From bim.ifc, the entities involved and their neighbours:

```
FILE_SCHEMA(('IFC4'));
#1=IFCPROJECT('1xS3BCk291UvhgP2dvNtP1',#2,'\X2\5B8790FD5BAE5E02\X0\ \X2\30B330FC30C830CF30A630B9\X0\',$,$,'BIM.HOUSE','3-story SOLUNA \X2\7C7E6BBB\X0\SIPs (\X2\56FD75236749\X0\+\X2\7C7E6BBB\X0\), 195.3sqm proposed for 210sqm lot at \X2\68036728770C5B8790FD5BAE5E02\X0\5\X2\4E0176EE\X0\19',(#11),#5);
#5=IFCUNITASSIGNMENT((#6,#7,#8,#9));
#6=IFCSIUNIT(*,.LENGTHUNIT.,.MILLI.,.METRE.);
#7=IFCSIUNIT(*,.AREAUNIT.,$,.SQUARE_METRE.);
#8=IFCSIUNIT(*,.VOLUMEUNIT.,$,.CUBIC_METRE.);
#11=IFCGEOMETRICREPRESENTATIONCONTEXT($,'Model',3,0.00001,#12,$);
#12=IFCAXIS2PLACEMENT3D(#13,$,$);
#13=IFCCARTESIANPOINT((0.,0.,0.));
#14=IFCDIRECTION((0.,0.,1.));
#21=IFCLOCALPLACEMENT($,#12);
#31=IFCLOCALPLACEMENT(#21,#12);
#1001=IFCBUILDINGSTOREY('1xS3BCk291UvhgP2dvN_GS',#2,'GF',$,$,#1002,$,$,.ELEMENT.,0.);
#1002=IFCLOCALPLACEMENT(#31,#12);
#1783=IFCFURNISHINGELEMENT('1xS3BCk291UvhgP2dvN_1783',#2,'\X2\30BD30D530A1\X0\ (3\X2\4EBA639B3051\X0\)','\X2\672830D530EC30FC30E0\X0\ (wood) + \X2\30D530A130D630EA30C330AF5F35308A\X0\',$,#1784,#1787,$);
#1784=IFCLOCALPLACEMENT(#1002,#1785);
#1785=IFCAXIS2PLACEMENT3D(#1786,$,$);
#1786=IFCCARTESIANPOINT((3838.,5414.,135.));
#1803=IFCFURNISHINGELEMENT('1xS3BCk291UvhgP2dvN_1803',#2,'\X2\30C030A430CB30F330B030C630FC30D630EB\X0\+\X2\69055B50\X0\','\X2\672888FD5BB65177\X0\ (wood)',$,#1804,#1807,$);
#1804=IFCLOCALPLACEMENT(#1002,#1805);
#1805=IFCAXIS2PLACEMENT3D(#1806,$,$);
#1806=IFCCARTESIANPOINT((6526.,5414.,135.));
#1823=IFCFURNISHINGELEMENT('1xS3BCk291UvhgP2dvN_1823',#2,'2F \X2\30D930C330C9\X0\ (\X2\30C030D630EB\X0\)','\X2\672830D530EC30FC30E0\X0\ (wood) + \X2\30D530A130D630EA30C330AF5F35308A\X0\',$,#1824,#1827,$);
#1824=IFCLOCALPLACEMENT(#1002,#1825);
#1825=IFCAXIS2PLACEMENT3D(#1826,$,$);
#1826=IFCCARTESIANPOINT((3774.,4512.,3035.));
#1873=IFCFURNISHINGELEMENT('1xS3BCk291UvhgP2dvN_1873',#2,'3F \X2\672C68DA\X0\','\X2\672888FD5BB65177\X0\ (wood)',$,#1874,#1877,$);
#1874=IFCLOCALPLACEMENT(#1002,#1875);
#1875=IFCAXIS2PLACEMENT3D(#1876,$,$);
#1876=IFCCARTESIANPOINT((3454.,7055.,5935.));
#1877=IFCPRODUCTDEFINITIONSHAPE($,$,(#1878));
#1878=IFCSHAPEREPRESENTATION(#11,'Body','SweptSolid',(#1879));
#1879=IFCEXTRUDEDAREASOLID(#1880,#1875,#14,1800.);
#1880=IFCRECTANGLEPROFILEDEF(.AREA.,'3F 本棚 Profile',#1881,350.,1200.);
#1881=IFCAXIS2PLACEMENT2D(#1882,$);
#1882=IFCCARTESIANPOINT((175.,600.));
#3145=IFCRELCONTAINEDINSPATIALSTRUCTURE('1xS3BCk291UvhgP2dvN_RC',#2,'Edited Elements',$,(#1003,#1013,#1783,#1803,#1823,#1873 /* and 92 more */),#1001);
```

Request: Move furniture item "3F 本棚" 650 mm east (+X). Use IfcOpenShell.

```python
import ifcopenshell
import ifcopenshell.api.geometry
import ifcopenshell.util.placement
import ifcopenshell.util.unit

model = ifcopenshell.open("bim.ifc")
unit_scale = ifcopenshell.util.unit.calculate_unit_scale(model)

item = model.by_id(1873)
matrix = ifcopenshell.util.placement.get_local_placement(item.ObjectPlacement)
matrix[0, 3] += 0.65 / unit_scale
ifcopenshell.api.geometry.edit_object_placement(model, product=item, matrix=matrix, is_si=False)

print(ifcopenshell.util.placement.get_local_placement(item.ObjectPlacement).round(3) + 0.0)

model.write("bim_v2.ifc")
```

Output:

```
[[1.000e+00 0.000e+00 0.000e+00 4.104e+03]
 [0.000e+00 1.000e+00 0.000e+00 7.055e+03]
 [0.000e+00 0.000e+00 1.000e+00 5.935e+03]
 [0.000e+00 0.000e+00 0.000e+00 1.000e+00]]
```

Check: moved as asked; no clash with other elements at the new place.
